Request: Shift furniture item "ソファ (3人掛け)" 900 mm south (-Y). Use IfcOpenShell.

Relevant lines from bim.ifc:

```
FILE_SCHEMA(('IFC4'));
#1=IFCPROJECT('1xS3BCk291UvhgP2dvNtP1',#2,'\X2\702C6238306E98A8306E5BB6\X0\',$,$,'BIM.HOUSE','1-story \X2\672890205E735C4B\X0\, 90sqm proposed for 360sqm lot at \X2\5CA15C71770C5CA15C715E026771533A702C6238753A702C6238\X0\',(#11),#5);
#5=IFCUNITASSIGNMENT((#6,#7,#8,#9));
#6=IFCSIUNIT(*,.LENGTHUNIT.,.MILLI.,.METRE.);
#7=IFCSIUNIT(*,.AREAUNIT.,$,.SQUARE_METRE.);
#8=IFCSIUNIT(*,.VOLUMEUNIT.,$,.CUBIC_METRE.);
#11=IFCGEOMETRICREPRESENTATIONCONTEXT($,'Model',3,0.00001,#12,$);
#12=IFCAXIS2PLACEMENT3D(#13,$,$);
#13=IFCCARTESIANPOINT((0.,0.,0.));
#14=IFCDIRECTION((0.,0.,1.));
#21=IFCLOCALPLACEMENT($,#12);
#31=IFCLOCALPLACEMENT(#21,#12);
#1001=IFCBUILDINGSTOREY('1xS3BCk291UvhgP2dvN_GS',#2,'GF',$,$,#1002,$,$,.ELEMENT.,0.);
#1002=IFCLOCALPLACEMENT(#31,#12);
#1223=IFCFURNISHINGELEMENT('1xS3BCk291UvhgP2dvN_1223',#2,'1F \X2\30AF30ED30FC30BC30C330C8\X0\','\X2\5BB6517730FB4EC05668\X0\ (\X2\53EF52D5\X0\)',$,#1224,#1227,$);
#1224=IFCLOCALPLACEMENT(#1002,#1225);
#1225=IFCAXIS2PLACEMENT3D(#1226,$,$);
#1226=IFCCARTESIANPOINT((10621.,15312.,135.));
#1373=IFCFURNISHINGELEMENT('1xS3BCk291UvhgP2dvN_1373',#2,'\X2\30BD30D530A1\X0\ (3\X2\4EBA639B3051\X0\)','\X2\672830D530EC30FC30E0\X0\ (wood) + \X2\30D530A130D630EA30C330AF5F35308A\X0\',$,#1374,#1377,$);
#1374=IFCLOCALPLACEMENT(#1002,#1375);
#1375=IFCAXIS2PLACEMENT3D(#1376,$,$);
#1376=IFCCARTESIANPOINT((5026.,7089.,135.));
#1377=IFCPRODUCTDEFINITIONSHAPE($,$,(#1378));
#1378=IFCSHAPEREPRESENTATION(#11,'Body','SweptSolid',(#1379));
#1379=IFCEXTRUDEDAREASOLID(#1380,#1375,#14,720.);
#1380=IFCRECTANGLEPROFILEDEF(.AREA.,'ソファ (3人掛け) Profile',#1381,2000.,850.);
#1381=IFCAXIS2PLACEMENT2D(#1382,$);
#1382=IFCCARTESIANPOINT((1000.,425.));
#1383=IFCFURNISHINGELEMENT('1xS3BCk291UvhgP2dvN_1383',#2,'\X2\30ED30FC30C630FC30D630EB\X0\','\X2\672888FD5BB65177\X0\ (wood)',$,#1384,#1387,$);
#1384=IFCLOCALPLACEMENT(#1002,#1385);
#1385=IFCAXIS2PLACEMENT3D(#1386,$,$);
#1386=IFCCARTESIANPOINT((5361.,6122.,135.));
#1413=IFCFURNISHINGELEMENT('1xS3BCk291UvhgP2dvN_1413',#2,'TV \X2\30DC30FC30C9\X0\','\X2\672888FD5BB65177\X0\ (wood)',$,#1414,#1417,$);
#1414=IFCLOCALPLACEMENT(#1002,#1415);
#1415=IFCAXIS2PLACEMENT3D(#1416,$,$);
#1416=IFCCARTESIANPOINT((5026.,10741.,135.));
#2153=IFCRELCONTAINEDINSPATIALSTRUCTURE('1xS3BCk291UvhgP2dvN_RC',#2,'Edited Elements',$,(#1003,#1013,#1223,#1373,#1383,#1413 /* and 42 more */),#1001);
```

```python
import ifcopenshell
import ifcopenshell.api.geometry
import ifcopenshell.util.placement
import ifcopenshell.util.unit

model = ifcopenshell.open("bim.ifc")
unit_scale = ifcopenshell.util.unit.calculate_unit_scale(model)

item = model.by_guid("1xS3BCk291UvhgP2dvN_1373")
matrix = ifcopenshell.util.placement.get_local_placement(item.ObjectPlacement)
matrix[1, 3] -= 0.9 / unit_scale
ifcopenshell.api.geometry.edit_object_placement(model, product=item, matrix=matrix, is_si=False)

print(ifcopenshell.util.placement.get_local_placement(item.ObjectPlacement).round(3) + 0.0)

model.write("bim_rev.ifc")
```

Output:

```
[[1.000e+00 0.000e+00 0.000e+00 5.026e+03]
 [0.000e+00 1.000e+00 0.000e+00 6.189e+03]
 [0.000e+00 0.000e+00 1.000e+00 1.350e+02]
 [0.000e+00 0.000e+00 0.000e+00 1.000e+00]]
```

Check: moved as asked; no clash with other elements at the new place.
